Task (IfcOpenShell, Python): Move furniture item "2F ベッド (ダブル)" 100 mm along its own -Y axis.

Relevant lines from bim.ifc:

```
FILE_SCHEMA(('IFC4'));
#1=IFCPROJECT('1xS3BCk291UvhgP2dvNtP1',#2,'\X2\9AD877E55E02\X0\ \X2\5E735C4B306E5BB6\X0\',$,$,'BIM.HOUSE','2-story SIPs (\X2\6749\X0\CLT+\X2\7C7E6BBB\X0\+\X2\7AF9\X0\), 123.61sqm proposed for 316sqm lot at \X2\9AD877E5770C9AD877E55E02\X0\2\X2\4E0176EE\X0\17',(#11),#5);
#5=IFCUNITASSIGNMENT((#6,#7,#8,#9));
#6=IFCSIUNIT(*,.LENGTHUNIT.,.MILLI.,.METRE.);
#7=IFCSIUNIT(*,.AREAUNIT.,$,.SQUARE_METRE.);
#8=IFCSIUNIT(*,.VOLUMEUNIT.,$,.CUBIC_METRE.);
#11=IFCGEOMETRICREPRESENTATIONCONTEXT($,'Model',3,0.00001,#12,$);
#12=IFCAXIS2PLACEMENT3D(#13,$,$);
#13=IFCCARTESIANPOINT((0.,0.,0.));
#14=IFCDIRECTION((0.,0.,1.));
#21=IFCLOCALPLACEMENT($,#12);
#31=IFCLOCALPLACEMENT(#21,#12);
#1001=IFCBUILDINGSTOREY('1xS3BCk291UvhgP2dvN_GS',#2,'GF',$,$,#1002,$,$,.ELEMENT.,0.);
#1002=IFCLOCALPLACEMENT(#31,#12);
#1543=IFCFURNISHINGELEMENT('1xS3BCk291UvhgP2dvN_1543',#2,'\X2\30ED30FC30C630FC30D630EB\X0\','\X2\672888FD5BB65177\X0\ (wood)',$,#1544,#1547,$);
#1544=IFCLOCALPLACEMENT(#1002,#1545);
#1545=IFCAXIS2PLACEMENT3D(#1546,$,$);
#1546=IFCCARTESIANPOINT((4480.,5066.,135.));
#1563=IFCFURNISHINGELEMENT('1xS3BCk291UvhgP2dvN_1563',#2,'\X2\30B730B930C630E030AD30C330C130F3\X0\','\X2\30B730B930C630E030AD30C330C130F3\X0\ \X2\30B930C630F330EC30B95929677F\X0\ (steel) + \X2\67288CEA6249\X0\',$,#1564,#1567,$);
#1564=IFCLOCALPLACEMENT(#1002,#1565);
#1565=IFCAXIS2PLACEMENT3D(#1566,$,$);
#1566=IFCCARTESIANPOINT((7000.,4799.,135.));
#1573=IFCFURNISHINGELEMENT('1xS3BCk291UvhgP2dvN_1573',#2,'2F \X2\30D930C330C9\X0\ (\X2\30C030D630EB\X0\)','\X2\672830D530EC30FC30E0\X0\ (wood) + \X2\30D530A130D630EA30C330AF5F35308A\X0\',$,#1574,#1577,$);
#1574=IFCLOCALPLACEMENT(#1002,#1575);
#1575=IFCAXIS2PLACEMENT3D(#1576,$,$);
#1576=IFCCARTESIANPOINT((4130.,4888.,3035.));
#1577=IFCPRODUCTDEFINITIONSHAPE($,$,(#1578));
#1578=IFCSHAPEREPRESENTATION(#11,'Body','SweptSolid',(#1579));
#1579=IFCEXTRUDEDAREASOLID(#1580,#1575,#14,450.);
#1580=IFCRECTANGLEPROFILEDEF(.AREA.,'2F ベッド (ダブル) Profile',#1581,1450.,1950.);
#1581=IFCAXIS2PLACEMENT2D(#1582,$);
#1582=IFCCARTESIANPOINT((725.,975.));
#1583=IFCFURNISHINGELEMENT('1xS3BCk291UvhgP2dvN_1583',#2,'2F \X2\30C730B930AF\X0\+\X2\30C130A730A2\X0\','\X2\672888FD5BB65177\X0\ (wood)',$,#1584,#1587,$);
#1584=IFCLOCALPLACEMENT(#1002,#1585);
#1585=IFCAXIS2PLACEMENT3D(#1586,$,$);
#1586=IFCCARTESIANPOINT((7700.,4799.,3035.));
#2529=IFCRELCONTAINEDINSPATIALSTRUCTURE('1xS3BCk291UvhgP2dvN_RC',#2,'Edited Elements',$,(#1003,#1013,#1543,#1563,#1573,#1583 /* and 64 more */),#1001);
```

```python
import ifcopenshell
import ifcopenshell.api.geometry
import ifcopenshell.util.placement
import ifcopenshell.util.unit

model = ifcopenshell.open("bim.ifc")
unit_scale = ifcopenshell.util.unit.calculate_unit_scale(model)

item = model.by_guid("1xS3BCk291UvhgP2dvN_1573")
matrix = ifcopenshell.util.placement.get_local_placement(item.ObjectPlacement)
matrix[:3, 3] -= matrix[:3, 1] * 0.1 / unit_scale
ifcopenshell.api.geometry.edit_object_placement(model, product=item, matrix=matrix, is_si=False)

print(ifcopenshell.util.placement.get_local_placement(item.ObjectPlacement).round(3) + 0.0)

model.write("bim_rev.ifc")
```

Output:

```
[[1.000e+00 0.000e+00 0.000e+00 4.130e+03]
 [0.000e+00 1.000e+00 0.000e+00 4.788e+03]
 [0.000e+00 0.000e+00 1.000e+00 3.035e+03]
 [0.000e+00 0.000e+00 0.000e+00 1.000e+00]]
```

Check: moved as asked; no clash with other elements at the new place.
